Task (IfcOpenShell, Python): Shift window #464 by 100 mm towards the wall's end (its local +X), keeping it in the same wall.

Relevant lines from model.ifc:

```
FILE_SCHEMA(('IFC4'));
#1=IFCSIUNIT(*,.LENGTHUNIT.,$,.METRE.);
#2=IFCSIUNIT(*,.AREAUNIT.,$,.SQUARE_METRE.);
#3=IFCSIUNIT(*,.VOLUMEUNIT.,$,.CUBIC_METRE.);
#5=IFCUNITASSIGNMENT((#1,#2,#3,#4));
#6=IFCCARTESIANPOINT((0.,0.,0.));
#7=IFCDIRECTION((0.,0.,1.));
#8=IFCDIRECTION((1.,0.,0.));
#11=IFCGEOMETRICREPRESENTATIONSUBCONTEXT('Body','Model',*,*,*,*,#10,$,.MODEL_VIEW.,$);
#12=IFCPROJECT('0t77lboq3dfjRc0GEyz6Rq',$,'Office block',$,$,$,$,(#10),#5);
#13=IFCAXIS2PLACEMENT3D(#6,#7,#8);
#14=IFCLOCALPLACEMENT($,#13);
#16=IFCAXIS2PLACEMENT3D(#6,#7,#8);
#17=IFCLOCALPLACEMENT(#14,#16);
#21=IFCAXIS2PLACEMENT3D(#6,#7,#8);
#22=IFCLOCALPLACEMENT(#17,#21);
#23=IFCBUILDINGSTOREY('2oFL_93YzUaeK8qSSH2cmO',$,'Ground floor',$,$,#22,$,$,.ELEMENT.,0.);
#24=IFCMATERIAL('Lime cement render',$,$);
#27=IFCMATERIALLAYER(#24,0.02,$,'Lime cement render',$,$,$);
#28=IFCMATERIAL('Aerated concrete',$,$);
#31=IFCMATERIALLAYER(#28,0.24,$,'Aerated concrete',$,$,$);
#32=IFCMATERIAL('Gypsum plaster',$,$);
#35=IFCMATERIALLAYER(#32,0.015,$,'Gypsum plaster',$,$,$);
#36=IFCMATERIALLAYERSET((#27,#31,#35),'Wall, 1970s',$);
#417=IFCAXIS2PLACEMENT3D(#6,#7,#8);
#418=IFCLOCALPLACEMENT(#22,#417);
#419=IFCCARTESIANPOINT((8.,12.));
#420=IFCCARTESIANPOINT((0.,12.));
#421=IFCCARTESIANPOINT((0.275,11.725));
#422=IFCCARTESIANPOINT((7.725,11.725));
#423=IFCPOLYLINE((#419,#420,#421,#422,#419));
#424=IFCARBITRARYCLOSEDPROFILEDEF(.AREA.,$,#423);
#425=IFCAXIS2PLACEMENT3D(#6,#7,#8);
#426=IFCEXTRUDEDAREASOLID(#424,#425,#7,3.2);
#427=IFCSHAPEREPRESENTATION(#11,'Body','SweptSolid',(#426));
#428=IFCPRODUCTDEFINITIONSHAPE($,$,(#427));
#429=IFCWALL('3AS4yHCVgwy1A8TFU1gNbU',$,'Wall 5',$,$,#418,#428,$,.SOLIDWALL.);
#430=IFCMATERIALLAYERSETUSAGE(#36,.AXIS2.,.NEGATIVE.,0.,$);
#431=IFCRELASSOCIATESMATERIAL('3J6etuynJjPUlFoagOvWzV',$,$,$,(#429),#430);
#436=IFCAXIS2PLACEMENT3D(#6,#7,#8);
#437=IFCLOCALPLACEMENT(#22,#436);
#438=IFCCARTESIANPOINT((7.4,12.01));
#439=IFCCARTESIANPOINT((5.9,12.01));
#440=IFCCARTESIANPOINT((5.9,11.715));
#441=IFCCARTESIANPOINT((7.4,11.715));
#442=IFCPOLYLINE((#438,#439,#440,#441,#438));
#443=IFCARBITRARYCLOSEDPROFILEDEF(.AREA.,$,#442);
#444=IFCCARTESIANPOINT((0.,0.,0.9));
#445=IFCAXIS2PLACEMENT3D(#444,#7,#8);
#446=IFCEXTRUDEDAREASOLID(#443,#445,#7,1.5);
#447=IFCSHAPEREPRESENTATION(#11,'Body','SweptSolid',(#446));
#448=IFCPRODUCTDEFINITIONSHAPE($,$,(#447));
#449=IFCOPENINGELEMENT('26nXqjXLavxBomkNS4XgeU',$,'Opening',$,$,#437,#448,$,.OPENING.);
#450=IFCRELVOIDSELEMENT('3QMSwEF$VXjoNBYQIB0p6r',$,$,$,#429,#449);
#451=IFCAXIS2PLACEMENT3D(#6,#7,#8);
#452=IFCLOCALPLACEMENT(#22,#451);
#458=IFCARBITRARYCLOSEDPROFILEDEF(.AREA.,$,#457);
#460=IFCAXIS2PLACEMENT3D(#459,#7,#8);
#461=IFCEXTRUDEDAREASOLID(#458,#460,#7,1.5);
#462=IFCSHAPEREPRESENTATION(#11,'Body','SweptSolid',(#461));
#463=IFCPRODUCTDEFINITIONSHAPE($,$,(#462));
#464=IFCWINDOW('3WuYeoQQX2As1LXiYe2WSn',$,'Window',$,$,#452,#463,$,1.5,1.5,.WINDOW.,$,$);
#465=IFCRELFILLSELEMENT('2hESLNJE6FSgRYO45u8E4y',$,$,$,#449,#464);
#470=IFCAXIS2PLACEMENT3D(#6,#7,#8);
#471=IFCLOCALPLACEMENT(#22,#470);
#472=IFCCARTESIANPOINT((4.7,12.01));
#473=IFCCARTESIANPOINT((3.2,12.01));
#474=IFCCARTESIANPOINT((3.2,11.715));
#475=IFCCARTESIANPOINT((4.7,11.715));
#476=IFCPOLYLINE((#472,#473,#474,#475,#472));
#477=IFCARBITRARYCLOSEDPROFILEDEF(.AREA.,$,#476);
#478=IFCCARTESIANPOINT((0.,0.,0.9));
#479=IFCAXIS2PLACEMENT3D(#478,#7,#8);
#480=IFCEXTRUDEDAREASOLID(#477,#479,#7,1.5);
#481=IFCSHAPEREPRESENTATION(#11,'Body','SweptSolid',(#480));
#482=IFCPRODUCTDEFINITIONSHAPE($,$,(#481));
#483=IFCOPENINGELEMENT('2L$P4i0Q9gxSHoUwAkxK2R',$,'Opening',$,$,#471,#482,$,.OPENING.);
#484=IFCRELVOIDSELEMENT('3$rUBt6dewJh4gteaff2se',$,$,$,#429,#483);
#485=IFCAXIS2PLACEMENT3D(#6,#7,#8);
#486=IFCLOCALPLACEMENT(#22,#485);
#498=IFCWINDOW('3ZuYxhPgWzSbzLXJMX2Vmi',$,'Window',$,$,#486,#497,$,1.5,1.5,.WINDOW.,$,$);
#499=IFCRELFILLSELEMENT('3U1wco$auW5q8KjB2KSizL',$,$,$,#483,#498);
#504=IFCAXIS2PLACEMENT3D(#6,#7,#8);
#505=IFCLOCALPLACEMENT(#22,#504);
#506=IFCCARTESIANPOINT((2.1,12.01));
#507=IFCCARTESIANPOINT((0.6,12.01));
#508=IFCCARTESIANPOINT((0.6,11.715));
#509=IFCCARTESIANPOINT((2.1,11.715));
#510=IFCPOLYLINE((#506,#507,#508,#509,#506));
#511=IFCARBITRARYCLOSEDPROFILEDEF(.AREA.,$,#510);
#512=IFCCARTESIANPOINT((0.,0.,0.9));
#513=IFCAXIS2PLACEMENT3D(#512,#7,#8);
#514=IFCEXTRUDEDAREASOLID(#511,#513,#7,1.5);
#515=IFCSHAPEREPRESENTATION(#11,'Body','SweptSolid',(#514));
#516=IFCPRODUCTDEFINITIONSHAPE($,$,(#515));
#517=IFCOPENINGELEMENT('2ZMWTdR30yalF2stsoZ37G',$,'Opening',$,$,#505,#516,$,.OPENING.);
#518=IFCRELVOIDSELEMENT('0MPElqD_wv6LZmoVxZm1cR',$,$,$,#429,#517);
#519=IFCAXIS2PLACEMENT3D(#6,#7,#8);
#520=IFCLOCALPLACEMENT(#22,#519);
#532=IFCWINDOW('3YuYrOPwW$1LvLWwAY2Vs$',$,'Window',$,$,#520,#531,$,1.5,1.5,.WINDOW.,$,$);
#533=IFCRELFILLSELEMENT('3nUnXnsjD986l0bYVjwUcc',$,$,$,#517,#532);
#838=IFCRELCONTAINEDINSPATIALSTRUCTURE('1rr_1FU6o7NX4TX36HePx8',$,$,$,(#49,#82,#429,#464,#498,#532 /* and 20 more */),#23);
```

```python
import ifcopenshell
import ifcopenshell.api.geometry
import ifcopenshell.util.placement
import ifcopenshell.util.unit

model = ifcopenshell.open("model.ifc")
unit_scale = ifcopenshell.util.unit.calculate_unit_scale(model)

window = model.by_id(464)
opening = window.FillsVoids[0].RelatingOpeningElement
wall = opening.VoidsElements[0].RelatingBuildingElement

wall_matrix = ifcopenshell.util.placement.get_local_placement(wall.ObjectPlacement)
shift = wall_matrix[:3, 0] * 0.1 / unit_scale
before = ifcopenshell.util.placement.get_local_placement(window.ObjectPlacement)[:3, 3].copy()

# The window is not placed relative to its opening, so move both.
for product in (opening, window):
    matrix = ifcopenshell.util.placement.get_local_placement(product.ObjectPlacement)
    matrix[:3, 3] += shift
    ifcopenshell.api.geometry.edit_object_placement(model, product=product, matrix=matrix, is_si=False)

after = ifcopenshell.util.placement.get_local_placement(window.ObjectPlacement)[:3, 3]
print("window moved by", (after - before).round(3) + 0.0)

model.write("model_v2.ifc")
```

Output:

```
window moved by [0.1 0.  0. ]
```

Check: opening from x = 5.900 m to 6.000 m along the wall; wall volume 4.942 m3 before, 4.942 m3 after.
